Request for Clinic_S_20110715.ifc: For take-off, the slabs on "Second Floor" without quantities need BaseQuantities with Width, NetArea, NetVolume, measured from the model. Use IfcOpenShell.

First a look at what the model holds.

```python
import ifcopenshell
import ifcopenshell.util.element
import ifcopenshell.util.unit

model = ifcopenshell.open("Clinic_S_20110715.ifc")
print(model.schema)
for unit_type in ("LENGTHUNIT", "AREAUNIT", "VOLUMEUNIT"):
    print(unit_type, ifcopenshell.util.unit.calculate_unit_scale(model, unit_type))
storey = next(s for s in model.by_type("IfcBuildingStorey") if s.Name == "Second Floor")
slabs = [e for e in ifcopenshell.util.element.get_decomposition(storey) if e.is_a("IfcSlab")]
for e in sorted(slabs, key=lambda e: e.id()):
    print(e.id(), e.is_a(), e.Name, list(ifcopenshell.util.element.get_psets(e, qtos_only=True)), sep=" | ")
```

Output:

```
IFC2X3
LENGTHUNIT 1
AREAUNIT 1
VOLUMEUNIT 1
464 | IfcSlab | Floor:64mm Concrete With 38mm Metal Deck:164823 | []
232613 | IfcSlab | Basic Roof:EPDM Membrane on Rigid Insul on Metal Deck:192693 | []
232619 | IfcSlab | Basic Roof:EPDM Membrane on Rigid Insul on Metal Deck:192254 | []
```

```python
import ifcopenshell
import ifcopenshell.api.pset
import ifcopenshell.geom
import ifcopenshell.util.element
import ifcopenshell.util.shape
import ifcopenshell.util.unit

model = ifcopenshell.open("Clinic_S_20110715.ifc")
unit_scale = ifcopenshell.util.unit.calculate_unit_scale(model)
area_scale = ifcopenshell.util.unit.calculate_unit_scale(model, "AREAUNIT")
volume_scale = ifcopenshell.util.unit.calculate_unit_scale(model, "VOLUMEUNIT")
settings = ifcopenshell.geom.settings()

storey = next(s for s in model.by_type("IfcBuildingStorey") if s.Name == "Second Floor")
slabs = [e for e in ifcopenshell.util.element.get_decomposition(storey) if e.is_a("IfcSlab")]

for e in sorted(slabs, key=lambda e: e.id()):
    if ifcopenshell.util.element.get_psets(e, qtos_only=True, should_inherit=False):
        continue
    # Geometry comes back in metres, in the element's own axes.
    shape = ifcopenshell.geom.create_shape(settings, e)
    values = {
        "Width": ifcopenshell.util.shape.get_z(shape.geometry) / unit_scale,
        "NetArea": ifcopenshell.util.shape.get_footprint_area(shape.geometry) / area_scale,
        "NetVolume": ifcopenshell.util.shape.get_volume(shape.geometry) / volume_scale,
    }
    qto = ifcopenshell.api.pset.add_qto(model, product=e, name="BaseQuantities")
    ifcopenshell.api.pset.edit_qto(model, qto=qto, properties=values)
    print(e.id(), {k: round(v, 3) for k, v in values.items()})

model.write("Clinic_S_20110715_edited.ifc")
```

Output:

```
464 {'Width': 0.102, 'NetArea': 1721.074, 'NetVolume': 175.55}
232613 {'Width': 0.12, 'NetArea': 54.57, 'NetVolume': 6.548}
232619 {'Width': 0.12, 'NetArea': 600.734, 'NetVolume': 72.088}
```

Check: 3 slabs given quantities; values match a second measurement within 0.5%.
